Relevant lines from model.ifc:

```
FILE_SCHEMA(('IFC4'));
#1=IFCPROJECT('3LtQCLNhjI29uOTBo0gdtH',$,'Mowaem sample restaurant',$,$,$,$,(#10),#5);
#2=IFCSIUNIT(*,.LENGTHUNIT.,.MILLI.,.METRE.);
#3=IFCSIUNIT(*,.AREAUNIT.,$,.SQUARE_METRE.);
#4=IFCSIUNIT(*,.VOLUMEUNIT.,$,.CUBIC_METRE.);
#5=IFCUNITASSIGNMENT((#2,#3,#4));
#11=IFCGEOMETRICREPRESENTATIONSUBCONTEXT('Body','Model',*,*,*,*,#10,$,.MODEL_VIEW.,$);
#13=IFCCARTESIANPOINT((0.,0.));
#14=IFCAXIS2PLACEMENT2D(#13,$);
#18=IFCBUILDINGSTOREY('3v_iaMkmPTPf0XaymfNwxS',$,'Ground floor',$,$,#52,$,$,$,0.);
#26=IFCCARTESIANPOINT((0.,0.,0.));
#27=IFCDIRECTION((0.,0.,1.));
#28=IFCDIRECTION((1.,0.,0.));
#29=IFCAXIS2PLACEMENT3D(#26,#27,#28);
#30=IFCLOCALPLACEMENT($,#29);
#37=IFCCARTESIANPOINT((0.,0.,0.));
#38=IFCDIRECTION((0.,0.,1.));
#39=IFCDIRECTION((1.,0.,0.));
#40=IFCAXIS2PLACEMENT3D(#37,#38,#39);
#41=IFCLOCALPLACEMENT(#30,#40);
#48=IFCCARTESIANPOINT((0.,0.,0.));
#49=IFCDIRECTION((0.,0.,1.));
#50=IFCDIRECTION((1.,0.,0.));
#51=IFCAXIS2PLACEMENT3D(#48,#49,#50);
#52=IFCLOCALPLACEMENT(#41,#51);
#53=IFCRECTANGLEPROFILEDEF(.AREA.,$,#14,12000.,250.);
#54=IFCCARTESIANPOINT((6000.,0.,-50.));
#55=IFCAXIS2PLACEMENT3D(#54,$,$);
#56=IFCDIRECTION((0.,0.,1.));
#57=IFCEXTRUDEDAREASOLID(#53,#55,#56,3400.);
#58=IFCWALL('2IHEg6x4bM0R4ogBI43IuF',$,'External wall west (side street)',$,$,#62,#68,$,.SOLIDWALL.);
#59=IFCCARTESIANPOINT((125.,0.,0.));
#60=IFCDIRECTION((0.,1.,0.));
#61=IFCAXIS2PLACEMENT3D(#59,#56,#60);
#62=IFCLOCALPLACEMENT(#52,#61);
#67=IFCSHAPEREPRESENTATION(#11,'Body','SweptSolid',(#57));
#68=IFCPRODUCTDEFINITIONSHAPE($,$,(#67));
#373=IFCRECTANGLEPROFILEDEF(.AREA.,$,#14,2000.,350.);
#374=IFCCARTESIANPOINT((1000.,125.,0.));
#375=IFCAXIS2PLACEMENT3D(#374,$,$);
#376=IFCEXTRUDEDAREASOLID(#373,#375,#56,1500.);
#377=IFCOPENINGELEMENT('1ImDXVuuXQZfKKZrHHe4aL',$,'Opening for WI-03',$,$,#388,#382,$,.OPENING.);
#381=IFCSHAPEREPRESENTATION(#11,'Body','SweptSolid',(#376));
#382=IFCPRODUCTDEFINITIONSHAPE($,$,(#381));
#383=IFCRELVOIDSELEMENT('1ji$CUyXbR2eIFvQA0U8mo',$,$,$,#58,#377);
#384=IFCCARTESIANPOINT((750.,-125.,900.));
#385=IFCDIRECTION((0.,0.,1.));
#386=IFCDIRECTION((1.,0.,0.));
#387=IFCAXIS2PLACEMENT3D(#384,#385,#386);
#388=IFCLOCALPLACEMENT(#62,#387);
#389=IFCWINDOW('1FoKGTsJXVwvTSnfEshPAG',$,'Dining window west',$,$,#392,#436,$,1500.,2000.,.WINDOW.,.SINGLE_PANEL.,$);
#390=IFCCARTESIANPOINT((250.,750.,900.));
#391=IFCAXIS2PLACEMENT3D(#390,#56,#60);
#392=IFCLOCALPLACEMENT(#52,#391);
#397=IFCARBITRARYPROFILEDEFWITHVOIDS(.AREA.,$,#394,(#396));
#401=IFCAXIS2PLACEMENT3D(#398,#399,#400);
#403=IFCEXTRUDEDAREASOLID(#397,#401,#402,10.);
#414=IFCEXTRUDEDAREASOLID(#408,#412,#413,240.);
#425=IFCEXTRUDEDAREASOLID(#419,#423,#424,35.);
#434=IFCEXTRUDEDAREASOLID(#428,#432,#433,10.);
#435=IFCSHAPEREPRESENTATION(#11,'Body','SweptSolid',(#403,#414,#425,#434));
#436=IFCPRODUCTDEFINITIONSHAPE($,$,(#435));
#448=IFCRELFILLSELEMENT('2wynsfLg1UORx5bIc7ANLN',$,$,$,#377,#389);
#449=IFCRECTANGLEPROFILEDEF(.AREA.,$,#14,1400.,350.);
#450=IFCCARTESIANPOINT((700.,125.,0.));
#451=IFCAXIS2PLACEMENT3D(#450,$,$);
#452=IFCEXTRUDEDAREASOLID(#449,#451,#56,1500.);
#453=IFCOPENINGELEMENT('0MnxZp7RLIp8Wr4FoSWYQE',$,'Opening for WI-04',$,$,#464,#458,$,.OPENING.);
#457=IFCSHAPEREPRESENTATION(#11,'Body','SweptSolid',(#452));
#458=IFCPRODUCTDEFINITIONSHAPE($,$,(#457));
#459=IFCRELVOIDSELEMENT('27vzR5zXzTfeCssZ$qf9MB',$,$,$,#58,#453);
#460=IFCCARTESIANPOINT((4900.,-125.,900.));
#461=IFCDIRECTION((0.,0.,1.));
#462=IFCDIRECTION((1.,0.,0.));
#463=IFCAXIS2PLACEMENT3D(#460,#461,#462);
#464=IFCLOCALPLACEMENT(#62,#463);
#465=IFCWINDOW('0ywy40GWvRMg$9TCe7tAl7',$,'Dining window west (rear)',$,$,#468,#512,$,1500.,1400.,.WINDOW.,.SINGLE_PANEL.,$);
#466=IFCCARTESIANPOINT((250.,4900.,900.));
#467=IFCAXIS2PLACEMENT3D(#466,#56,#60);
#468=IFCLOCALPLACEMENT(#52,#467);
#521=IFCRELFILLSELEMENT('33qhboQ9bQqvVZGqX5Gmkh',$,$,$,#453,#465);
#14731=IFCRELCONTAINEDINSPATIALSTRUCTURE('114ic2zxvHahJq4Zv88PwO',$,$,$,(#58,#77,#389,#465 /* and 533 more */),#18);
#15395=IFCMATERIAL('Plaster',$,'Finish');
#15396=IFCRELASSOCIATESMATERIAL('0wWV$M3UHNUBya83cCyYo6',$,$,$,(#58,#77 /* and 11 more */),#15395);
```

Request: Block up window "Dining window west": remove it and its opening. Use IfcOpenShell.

```python
import ifcopenshell
import ifcopenshell.api.feature
import ifcopenshell.api.root
import ifcopenshell.geom
import ifcopenshell.util.shape

model = ifcopenshell.open("model.ifc")
settings = ifcopenshell.geom.settings()


def volume(element):
    """Net volume in cubic metres, openings subtracted."""
    shape = ifcopenshell.geom.create_shape(settings, element)
    return ifcopenshell.util.shape.get_volume(shape.geometry)


window = model.by_id(389)
opening = window.FillsVoids[0].RelatingOpeningElement
wall = opening.VoidsElements[0].RelatingBuildingElement
before = volume(wall)

ifcopenshell.api.root.remove_product(model, product=window)
ifcopenshell.api.feature.remove_feature(model, feature=opening)

after = volume(wall)

print(f"wall volume {before:.3f} -> {after:.3f} m3")

model.write("model_v2.ifc")
```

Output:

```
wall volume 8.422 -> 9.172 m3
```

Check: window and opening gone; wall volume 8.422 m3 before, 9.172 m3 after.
